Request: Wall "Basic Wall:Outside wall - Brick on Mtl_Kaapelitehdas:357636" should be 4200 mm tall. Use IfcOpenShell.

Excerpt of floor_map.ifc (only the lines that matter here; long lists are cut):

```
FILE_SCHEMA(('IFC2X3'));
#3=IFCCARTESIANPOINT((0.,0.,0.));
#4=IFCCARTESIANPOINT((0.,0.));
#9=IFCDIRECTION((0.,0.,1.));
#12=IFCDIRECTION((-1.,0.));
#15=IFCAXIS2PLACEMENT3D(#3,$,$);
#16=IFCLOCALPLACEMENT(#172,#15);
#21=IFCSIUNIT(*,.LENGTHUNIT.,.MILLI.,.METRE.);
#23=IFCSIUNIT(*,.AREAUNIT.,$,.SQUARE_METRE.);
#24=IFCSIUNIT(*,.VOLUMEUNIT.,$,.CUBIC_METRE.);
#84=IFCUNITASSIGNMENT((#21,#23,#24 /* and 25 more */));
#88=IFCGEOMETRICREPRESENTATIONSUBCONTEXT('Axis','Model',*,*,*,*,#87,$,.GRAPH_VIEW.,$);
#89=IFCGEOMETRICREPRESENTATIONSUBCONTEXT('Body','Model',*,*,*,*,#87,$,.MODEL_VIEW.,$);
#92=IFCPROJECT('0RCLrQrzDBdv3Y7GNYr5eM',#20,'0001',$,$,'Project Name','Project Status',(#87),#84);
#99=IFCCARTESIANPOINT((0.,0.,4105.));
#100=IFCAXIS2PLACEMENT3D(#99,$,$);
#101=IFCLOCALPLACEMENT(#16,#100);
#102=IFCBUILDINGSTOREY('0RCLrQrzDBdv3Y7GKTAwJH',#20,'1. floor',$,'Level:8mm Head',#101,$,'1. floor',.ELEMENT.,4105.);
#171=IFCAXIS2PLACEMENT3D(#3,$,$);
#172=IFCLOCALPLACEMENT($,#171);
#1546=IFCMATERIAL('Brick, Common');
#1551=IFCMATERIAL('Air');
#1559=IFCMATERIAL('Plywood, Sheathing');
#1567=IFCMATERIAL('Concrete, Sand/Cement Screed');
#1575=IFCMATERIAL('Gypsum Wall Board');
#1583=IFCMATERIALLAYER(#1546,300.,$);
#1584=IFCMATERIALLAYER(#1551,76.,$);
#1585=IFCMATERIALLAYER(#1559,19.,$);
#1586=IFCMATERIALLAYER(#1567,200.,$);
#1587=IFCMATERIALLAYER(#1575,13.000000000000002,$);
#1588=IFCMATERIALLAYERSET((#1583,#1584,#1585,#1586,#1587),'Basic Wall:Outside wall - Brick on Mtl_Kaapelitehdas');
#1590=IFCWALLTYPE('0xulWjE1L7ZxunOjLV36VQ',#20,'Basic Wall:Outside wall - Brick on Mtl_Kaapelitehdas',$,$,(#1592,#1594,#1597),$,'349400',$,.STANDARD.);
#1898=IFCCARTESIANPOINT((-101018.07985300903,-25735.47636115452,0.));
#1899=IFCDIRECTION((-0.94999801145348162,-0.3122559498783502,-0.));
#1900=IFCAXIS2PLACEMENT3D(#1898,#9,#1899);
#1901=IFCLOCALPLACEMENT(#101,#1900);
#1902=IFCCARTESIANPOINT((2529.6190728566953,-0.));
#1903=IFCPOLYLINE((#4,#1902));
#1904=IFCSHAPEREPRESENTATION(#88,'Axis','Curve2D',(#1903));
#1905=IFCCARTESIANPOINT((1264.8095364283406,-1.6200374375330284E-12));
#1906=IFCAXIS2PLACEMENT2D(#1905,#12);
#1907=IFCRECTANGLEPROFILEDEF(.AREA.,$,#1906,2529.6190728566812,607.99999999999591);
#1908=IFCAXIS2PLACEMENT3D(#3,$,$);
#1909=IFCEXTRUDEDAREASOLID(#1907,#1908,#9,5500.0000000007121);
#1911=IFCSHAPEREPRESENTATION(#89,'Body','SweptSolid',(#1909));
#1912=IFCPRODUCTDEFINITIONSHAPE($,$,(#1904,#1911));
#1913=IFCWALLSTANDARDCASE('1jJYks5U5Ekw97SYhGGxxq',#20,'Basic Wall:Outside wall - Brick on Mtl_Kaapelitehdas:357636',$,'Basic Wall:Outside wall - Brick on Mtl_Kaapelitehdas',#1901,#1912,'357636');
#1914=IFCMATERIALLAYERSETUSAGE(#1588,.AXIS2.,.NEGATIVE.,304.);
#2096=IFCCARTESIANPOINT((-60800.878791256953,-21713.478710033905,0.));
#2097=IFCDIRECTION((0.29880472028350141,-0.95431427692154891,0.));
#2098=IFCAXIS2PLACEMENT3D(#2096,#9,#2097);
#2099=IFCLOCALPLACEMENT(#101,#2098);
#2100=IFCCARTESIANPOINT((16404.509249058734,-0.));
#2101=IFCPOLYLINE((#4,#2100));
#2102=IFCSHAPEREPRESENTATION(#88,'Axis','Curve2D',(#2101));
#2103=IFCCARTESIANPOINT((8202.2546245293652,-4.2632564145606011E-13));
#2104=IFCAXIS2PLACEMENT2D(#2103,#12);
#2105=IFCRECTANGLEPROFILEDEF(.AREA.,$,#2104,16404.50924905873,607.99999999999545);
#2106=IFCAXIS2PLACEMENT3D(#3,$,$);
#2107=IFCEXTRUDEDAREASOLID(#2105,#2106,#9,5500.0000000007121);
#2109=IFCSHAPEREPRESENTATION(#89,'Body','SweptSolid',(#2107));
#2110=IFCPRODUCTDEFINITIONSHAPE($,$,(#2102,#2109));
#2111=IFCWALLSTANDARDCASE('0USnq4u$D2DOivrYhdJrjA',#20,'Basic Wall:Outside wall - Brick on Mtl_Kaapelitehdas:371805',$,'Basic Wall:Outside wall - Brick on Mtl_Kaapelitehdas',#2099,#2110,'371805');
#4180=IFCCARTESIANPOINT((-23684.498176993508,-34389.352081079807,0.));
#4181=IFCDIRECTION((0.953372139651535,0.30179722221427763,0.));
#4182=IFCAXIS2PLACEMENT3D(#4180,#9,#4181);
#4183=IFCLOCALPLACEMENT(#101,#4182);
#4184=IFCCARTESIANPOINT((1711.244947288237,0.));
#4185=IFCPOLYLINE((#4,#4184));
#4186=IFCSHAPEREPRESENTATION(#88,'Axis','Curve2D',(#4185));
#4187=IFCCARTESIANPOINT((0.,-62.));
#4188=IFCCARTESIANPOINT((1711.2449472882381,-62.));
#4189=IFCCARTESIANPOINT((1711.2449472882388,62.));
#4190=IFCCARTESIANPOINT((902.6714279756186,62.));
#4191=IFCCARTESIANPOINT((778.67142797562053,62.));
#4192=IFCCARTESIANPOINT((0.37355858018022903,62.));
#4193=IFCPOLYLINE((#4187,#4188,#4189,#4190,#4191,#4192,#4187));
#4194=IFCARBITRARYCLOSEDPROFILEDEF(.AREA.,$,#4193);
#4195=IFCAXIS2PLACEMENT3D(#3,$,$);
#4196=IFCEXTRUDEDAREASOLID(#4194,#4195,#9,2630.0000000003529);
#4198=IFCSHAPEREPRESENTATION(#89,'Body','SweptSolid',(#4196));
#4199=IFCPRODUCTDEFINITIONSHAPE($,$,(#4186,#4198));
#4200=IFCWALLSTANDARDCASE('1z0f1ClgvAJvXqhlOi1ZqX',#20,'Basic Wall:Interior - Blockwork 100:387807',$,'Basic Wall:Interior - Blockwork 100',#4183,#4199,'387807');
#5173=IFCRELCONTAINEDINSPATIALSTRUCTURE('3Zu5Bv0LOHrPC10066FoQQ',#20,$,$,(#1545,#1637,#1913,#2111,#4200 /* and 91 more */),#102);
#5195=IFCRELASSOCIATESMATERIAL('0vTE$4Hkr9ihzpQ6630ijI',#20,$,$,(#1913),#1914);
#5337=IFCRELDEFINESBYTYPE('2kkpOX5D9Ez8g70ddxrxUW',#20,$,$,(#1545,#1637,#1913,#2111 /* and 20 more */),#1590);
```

```python
import ifcopenshell
import ifcopenshell.geom
import ifcopenshell.util.representation
import ifcopenshell.util.shape

model = ifcopenshell.open("floor_map.ifc")
settings = ifcopenshell.geom.settings()


def volume(element):
    """Net volume in cubic metres, openings subtracted."""
    shape = ifcopenshell.geom.create_shape(settings, element)
    return ifcopenshell.util.shape.get_volume(shape.geometry)


wall = model.by_guid("1jJYks5U5Ekw97SYhGGxxq")
before = volume(wall)

body = ifcopenshell.util.representation.get_representation(wall, "Model", "Body")
solid = body.Items[0]
old_height = solid.Depth
solid.Depth = 4200.0
after = volume(wall)

print(f"height {old_height:g} -> {solid.Depth:g}, volume {before:.3f} -> {after:.3f} m3")

model.write("floor_map_updated.ifc")
```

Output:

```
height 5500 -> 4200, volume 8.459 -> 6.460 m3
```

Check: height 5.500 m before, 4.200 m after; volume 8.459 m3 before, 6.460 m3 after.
